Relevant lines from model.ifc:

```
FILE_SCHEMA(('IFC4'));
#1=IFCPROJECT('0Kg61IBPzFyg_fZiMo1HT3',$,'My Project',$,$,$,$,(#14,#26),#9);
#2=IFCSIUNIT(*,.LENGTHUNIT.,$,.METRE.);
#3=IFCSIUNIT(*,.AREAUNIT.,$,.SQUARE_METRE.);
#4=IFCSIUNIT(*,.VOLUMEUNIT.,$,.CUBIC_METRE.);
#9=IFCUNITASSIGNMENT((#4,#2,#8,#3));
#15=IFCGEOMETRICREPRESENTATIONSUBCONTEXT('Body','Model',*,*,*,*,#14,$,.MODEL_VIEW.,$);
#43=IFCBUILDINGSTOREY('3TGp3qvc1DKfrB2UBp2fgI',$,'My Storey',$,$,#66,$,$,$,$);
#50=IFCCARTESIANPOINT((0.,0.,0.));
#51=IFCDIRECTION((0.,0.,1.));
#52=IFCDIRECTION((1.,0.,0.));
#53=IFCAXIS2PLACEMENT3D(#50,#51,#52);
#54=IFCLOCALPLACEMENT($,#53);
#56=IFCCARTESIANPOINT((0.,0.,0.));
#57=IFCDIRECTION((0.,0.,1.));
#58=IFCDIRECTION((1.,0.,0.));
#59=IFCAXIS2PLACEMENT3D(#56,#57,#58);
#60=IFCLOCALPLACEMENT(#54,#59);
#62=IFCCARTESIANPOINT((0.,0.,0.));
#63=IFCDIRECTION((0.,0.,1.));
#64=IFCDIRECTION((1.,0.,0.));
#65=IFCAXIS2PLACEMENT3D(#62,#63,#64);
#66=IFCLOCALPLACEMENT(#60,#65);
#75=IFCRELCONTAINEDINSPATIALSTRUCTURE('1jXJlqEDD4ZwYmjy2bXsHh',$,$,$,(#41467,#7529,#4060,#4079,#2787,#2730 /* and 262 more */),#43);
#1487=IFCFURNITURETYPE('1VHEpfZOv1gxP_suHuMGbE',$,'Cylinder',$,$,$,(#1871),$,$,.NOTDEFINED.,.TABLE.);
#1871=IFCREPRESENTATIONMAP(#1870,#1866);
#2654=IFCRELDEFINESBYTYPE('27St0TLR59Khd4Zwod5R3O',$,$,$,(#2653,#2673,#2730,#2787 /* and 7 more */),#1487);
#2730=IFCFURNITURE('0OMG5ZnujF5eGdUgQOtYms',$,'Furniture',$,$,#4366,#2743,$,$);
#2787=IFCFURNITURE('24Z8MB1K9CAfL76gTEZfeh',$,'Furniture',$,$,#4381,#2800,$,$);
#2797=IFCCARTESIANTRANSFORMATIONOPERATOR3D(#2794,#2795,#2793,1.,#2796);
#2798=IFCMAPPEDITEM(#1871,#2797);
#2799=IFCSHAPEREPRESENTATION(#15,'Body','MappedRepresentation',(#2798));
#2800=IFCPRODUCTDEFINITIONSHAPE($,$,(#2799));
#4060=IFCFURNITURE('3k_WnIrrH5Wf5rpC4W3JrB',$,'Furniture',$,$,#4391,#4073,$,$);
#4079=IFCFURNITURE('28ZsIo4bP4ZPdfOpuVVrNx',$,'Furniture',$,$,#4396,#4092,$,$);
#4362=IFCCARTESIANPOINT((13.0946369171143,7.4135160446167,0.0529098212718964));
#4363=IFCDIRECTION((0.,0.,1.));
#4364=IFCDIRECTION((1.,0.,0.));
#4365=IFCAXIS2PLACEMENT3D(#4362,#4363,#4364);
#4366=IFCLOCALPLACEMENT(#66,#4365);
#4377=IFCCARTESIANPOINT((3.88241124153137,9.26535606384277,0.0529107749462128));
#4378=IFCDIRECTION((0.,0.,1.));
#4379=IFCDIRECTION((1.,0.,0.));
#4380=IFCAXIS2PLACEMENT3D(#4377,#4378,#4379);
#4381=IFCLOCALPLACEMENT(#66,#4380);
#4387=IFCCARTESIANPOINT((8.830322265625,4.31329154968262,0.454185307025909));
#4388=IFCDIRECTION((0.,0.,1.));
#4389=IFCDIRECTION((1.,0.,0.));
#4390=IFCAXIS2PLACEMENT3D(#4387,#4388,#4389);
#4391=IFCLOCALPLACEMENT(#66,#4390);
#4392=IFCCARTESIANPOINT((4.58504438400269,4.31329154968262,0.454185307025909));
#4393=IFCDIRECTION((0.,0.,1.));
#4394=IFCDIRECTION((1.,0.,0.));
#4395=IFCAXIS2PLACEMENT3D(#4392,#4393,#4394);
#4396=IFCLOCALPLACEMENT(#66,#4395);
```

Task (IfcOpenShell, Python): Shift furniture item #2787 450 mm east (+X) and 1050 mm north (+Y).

```python
import ifcopenshell
import ifcopenshell.api.geometry
import ifcopenshell.util.placement
import ifcopenshell.util.unit

model = ifcopenshell.open("model.ifc")
unit_scale = ifcopenshell.util.unit.calculate_unit_scale(model)

item = model.by_guid("24Z8MB1K9CAfL76gTEZfeh")
matrix = ifcopenshell.util.placement.get_local_placement(item.ObjectPlacement)
matrix[0, 3] += 0.45 / unit_scale
matrix[1, 3] += 1.05 / unit_scale
ifcopenshell.api.geometry.edit_object_placement(model, product=item, matrix=matrix, is_si=False)

print(ifcopenshell.util.placement.get_local_placement(item.ObjectPlacement).round(3) + 0.0)

model.write("model_rev.ifc")
```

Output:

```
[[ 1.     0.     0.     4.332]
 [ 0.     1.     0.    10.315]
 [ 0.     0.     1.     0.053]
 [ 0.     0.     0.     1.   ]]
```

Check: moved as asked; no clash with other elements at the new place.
